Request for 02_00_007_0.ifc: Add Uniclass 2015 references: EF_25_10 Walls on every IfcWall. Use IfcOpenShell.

First a look at what the model holds.

```python
import ifcopenshell

model = ifcopenshell.open("02_00_007_0.ifc")
print(model.schema)
print("classifications:", [c.Name for c in model.by_type("IfcClassification")])
for ifc_class in ("IfcDoor", "IfcRoof", "IfcStair", "IfcWall", "IfcWindow"):
    print(ifc_class, len(model.by_type(ifc_class)))
```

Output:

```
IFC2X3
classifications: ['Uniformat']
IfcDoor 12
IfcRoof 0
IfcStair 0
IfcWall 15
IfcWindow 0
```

```python
import ifcopenshell
import ifcopenshell.api.classification

model = ifcopenshell.open("02_00_007_0.ifc")

# IFC2X3 requires Source and Edition and has no link from the project to the system.
system = model.create_entity("IfcClassification", Source="NBS", Edition="2015", Name="Uniclass 2015")

codes = {
    "IfcWall": ("EF_25_10", "Walls"),
}
for ifc_class, (code, name) in codes.items():
    products = model.by_type(ifc_class)
    ifcopenshell.api.classification.add_reference(
        model, products=products, classification=system, identification=code, name=name
    )
    print(code, len(products))

model.write("02_00_007_0-out.ifc")
```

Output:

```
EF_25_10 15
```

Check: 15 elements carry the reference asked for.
